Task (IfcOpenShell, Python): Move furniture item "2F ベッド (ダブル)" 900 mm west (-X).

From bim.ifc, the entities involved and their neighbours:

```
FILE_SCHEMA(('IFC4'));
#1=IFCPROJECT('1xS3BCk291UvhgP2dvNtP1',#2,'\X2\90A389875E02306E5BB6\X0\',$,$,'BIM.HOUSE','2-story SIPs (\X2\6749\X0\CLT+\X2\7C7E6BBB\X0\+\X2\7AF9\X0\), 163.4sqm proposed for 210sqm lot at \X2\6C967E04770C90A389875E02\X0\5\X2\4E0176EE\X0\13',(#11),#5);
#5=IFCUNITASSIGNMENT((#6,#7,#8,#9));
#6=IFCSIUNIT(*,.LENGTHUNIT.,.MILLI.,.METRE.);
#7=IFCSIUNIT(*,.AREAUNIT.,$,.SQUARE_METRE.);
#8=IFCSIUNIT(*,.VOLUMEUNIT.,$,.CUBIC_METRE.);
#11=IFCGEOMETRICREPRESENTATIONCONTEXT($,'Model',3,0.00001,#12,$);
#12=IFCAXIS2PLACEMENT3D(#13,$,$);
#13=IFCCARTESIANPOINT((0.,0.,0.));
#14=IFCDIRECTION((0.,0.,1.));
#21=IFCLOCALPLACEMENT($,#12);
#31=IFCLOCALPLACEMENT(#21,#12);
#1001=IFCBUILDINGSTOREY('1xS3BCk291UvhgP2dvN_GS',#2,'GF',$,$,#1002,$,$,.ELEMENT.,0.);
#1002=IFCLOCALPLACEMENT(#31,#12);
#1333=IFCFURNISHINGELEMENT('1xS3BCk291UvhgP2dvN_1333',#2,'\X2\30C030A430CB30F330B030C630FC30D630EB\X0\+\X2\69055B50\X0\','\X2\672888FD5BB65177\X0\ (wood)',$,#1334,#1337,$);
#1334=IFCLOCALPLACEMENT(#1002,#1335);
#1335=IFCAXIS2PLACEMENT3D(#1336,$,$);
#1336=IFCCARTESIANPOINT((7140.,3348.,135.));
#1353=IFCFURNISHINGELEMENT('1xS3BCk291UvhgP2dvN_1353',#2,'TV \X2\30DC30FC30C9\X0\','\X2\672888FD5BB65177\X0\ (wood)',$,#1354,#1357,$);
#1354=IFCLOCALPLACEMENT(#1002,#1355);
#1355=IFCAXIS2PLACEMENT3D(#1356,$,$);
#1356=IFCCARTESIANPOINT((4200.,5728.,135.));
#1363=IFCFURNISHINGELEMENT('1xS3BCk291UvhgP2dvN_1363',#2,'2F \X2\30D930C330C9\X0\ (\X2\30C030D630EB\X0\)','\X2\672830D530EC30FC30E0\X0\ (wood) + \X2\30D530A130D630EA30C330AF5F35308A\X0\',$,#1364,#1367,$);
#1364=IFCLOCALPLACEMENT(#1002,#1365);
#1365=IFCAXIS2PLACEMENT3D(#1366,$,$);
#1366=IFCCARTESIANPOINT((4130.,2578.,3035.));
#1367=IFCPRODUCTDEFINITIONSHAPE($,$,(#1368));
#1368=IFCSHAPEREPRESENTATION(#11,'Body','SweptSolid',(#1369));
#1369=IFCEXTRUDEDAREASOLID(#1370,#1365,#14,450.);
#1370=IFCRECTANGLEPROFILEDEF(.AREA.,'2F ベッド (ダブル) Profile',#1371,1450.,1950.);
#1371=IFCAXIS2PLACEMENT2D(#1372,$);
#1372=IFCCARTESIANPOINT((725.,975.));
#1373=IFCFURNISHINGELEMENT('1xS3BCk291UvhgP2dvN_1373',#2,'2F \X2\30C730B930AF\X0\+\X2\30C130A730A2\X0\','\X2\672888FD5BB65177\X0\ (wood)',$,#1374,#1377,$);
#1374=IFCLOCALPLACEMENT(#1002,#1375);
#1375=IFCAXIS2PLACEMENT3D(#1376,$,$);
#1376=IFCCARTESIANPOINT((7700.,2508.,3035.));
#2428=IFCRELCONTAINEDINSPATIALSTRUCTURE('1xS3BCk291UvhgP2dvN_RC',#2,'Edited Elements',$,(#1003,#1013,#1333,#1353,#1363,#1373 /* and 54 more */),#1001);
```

```python
import ifcopenshell
import ifcopenshell.api.geometry
import ifcopenshell.util.placement
import ifcopenshell.util.unit

model = ifcopenshell.open("bim.ifc")
unit_scale = ifcopenshell.util.unit.calculate_unit_scale(model)

item = model.by_guid("1xS3BCk291UvhgP2dvN_1363")
matrix = ifcopenshell.util.placement.get_local_placement(item.ObjectPlacement)
matrix[0, 3] -= 0.9 / unit_scale
ifcopenshell.api.geometry.edit_object_placement(model, product=item, matrix=matrix, is_si=False)

print(ifcopenshell.util.placement.get_local_placement(item.ObjectPlacement).round(3) + 0.0)

model.write("bim-out.ifc")
```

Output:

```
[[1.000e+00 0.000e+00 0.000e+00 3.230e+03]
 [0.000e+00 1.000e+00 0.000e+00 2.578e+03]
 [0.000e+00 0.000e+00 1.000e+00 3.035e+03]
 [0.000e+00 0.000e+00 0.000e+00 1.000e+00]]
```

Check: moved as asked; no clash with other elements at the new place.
